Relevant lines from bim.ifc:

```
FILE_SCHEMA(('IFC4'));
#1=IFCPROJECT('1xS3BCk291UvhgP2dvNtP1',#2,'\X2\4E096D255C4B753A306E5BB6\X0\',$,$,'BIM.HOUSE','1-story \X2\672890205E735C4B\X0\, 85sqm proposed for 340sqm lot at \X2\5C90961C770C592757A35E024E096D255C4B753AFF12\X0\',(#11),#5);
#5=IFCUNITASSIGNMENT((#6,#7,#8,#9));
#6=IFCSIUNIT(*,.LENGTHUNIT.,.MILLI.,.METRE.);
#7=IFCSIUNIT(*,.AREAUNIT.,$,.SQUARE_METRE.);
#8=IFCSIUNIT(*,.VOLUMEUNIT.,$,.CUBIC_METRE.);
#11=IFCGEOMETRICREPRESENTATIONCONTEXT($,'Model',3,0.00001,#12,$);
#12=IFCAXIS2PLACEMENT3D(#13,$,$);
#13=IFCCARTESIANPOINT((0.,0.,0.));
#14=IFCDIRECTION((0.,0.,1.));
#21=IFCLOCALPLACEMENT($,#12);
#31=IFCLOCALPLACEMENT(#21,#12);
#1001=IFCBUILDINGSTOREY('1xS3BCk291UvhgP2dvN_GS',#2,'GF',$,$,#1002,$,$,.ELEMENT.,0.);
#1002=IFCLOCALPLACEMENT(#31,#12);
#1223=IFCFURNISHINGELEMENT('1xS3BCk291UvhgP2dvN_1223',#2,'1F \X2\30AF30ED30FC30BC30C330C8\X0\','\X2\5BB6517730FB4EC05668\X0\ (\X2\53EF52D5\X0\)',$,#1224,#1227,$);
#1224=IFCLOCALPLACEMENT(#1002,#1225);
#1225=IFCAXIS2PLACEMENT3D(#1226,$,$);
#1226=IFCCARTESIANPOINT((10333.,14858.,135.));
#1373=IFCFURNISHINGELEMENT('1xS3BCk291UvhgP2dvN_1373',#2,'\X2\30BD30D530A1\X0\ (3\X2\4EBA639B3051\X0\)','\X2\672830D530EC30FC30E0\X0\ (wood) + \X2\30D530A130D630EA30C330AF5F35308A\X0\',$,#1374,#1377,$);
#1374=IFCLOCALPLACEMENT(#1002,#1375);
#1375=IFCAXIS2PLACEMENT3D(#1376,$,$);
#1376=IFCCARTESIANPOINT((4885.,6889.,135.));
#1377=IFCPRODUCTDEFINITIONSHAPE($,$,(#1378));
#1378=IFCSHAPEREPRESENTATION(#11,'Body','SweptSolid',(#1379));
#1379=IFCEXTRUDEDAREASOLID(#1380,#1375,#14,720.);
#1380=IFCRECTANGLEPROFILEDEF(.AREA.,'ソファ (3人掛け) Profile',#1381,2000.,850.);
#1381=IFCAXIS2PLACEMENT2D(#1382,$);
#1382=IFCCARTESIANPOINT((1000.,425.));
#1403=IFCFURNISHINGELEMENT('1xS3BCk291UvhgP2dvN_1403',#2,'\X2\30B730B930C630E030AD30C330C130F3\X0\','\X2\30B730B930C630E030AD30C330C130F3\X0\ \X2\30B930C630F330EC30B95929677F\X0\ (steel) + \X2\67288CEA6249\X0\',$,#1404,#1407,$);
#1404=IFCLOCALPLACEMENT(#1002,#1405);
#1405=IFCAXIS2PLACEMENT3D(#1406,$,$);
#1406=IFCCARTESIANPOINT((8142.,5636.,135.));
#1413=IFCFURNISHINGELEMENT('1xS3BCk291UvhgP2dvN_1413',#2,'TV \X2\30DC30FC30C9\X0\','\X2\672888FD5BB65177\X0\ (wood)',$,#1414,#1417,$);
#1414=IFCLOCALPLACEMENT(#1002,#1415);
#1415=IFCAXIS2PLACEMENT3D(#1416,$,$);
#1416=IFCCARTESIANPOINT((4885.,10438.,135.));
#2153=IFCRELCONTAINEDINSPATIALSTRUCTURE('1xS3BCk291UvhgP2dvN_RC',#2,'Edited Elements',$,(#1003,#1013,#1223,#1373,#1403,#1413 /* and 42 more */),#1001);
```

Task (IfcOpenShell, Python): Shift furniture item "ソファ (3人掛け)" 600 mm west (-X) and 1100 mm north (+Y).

```python
import ifcopenshell
import ifcopenshell.api.geometry
import ifcopenshell.util.placement
import ifcopenshell.util.unit

model = ifcopenshell.open("bim.ifc")
unit_scale = ifcopenshell.util.unit.calculate_unit_scale(model)

item = model.by_guid("1xS3BCk291UvhgP2dvN_1373")
matrix = ifcopenshell.util.placement.get_local_placement(item.ObjectPlacement)
matrix[0, 3] -= 0.6 / unit_scale
matrix[1, 3] += 1.1 / unit_scale
ifcopenshell.api.geometry.edit_object_placement(model, product=item, matrix=matrix, is_si=False)

print(ifcopenshell.util.placement.get_local_placement(item.ObjectPlacement).round(3) + 0.0)

model.write("bim_edited.ifc")
```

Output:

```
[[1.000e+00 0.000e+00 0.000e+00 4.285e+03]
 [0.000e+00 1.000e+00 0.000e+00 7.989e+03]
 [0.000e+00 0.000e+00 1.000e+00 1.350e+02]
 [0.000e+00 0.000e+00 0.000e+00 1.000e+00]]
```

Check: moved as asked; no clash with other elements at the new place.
